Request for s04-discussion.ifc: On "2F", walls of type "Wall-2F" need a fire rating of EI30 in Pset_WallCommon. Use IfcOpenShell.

First a look at what the model holds.

```python
import ifcopenshell
import ifcopenshell.util.element

model = ifcopenshell.open("s04-discussion.ifc")
print(model.schema)
storey = next(s for s in model.by_type("IfcBuildingStorey") if s.Name == "2F")
walls = [e for e in ifcopenshell.util.element.get_decomposition(storey) if e.is_a("IfcWall")]
seen = {}
for e in walls:
    element_type = ifcopenshell.util.element.get_type(e)
    key = (element_type.Name if element_type != e and element_type else None, ifcopenshell.util.element.get_pset(e, "Pset_WallCommon", "FireRating"))
    seen[key] = seen.get(key, 0) + 1
for (name, value), count in sorted(seen.items(), key=str):
    print(count, "x", name, "|", value)
```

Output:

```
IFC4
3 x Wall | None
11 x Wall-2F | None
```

```python
import ifcopenshell
import ifcopenshell.api.pset
import ifcopenshell.util.element

model = ifcopenshell.open("s04-discussion.ifc")

storey = next(s for s in model.by_type("IfcBuildingStorey") if s.Name == "2F")
walls = [e for e in ifcopenshell.util.element.get_decomposition(storey) if e.is_a("IfcWall")]

count = 0
for e in walls:
    element_type = ifcopenshell.util.element.get_type(e)
    if element_type in (None, e) or element_type.Name != "Wall-2F":
        continue
    # add_pset returns the element's existing set when there is one.
    pset = ifcopenshell.api.pset.add_pset(model, product=e, name="Pset_WallCommon")
    ifcopenshell.api.pset.edit_pset(model, pset=pset, properties={"FireRating": "EI30"})
    count += 1

print(count, "walls updated")

model.write("s04-discussion_updated.ifc")
```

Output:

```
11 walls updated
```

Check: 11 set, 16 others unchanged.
